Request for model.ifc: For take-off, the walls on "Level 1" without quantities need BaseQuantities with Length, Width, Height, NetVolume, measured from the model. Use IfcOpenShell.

First a look at what the model holds.

```python
import ifcopenshell
import ifcopenshell.util.element
import ifcopenshell.util.unit

model = ifcopenshell.open("model.ifc")
print(model.schema)
for unit_type in ("LENGTHUNIT", "AREAUNIT", "VOLUMEUNIT"):
    print(unit_type, ifcopenshell.util.unit.calculate_unit_scale(model, unit_type))
storey = next(s for s in model.by_type("IfcBuildingStorey") if s.Name == "Level 1")
walls = [e for e in ifcopenshell.util.element.get_decomposition(storey) if e.is_a("IfcWall")]
for e in sorted(walls, key=lambda e: e.id()):
    print(e.id(), e.is_a(), e.Name, list(ifcopenshell.util.element.get_psets(e, qtos_only=True)), sep=" | ")
```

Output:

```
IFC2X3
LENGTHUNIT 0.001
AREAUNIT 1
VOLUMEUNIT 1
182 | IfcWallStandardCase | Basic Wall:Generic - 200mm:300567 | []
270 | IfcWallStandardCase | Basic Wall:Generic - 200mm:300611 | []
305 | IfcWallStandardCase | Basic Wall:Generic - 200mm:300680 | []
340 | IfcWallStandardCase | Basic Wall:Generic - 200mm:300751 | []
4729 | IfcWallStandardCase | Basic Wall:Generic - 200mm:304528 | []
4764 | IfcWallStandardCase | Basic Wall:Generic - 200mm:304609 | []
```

```python
import ifcopenshell
import ifcopenshell.api.pset
import ifcopenshell.geom
import ifcopenshell.util.element
import ifcopenshell.util.shape
import ifcopenshell.util.unit

model = ifcopenshell.open("model.ifc")
unit_scale = ifcopenshell.util.unit.calculate_unit_scale(model)
volume_scale = ifcopenshell.util.unit.calculate_unit_scale(model, "VOLUMEUNIT")
settings = ifcopenshell.geom.settings()

storey = next(s for s in model.by_type("IfcBuildingStorey") if s.Name == "Level 1")
walls = [e for e in ifcopenshell.util.element.get_decomposition(storey) if e.is_a("IfcWall")]

for e in sorted(walls, key=lambda e: e.id()):
    if ifcopenshell.util.element.get_psets(e, qtos_only=True, should_inherit=False):
        continue
    # Geometry comes back in metres, in the element's own axes.
    shape = ifcopenshell.geom.create_shape(settings, e)
    values = {
        "Length": ifcopenshell.util.shape.get_x(shape.geometry) / unit_scale,
        "Width": ifcopenshell.util.shape.get_y(shape.geometry) / unit_scale,
        "Height": ifcopenshell.util.shape.get_z(shape.geometry) / unit_scale,
        "NetVolume": ifcopenshell.util.shape.get_volume(shape.geometry) / volume_scale,
    }
    qto = ifcopenshell.api.pset.add_qto(model, product=e, name="BaseQuantities")
    ifcopenshell.api.pset.edit_qto(model, qto=qto, properties=values)
    print(e.id(), {k: round(v, 3) for k, v in values.items()})

model.write("model-out.ifc")
```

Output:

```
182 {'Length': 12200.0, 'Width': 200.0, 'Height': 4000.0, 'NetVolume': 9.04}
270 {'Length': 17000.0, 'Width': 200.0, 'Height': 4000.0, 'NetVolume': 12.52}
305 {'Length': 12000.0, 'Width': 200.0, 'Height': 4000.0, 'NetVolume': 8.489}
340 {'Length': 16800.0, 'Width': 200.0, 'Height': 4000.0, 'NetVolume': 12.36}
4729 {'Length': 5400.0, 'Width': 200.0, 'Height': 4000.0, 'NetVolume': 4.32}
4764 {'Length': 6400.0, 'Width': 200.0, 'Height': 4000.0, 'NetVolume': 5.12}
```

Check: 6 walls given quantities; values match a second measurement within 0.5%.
